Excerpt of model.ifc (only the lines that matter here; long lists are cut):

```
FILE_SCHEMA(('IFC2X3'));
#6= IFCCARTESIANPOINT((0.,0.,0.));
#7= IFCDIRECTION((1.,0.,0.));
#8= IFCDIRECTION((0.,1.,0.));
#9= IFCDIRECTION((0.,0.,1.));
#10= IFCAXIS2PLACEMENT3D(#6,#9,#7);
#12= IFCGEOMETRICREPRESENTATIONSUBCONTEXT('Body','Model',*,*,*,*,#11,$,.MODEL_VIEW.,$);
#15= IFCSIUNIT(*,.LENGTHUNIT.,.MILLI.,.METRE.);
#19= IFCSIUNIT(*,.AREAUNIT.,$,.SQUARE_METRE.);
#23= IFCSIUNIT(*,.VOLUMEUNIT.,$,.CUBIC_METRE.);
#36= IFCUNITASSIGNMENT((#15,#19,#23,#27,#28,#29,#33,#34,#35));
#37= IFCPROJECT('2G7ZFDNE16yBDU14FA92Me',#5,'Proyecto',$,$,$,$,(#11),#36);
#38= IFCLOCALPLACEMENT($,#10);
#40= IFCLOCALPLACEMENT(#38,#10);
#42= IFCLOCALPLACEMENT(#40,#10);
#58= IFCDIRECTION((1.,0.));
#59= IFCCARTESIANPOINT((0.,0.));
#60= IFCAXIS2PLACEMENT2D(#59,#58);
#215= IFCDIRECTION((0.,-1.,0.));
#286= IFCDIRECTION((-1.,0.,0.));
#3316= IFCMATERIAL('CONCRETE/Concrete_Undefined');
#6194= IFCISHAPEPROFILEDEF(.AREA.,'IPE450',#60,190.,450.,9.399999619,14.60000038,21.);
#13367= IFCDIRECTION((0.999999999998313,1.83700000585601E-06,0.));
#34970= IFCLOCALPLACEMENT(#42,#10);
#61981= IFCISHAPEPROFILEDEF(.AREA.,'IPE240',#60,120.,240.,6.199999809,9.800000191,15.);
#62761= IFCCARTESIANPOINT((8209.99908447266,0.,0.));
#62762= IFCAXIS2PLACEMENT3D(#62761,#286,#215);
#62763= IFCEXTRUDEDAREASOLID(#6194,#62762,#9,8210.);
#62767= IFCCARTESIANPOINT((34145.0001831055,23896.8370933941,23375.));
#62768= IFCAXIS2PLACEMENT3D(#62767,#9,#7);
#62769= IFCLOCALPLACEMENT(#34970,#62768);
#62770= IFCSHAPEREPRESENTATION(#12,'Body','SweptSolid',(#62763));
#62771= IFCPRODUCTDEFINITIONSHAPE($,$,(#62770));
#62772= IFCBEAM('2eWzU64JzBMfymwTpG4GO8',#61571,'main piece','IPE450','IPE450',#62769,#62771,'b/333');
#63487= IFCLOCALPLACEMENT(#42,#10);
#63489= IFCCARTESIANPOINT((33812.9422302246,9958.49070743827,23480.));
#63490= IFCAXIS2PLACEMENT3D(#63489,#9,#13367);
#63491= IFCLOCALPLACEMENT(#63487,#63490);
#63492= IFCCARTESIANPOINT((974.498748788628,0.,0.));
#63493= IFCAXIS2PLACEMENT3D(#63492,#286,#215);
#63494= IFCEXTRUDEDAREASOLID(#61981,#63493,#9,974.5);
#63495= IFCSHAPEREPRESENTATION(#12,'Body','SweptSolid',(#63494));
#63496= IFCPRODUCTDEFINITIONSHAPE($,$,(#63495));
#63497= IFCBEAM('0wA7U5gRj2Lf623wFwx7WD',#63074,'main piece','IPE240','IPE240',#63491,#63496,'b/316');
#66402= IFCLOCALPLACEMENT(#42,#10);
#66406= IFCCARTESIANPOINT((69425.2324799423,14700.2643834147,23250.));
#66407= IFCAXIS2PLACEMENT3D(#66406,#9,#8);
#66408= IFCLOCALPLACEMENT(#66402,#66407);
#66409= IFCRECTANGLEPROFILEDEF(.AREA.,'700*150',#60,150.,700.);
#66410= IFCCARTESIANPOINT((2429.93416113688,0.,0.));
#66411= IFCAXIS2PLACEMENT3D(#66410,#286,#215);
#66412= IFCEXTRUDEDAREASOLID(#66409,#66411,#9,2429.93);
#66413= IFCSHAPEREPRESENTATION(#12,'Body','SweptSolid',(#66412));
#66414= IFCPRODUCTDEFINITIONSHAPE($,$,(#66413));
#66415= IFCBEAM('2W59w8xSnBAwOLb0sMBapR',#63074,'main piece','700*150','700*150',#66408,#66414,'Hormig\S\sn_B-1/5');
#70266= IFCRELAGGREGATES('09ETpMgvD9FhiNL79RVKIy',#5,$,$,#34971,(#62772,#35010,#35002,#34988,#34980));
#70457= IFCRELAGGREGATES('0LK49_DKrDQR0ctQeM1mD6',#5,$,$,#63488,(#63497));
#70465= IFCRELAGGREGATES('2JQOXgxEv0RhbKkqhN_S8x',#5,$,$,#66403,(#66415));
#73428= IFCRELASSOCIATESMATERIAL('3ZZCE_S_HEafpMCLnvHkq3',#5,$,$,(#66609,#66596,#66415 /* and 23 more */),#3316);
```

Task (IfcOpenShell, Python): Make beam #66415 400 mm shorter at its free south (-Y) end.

```python
import ifcopenshell
import ifcopenshell.util.representation

model = ifcopenshell.open("model.ifc")

member = model.by_guid("2W59w8xSnBAwOLb0sMBapR")
change = -400.0

# The extrusion runs towards the end named, so only its depth changes.
body = ifcopenshell.util.representation.get_representation(member, "Model", "Body")
solid = body.Items[0]
old_length = solid.Depth
solid.Depth += change

print(f"length {old_length:g} -> {solid.Depth:g}")

model.write("model_v2.ifc")
```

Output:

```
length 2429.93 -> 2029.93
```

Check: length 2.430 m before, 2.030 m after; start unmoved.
